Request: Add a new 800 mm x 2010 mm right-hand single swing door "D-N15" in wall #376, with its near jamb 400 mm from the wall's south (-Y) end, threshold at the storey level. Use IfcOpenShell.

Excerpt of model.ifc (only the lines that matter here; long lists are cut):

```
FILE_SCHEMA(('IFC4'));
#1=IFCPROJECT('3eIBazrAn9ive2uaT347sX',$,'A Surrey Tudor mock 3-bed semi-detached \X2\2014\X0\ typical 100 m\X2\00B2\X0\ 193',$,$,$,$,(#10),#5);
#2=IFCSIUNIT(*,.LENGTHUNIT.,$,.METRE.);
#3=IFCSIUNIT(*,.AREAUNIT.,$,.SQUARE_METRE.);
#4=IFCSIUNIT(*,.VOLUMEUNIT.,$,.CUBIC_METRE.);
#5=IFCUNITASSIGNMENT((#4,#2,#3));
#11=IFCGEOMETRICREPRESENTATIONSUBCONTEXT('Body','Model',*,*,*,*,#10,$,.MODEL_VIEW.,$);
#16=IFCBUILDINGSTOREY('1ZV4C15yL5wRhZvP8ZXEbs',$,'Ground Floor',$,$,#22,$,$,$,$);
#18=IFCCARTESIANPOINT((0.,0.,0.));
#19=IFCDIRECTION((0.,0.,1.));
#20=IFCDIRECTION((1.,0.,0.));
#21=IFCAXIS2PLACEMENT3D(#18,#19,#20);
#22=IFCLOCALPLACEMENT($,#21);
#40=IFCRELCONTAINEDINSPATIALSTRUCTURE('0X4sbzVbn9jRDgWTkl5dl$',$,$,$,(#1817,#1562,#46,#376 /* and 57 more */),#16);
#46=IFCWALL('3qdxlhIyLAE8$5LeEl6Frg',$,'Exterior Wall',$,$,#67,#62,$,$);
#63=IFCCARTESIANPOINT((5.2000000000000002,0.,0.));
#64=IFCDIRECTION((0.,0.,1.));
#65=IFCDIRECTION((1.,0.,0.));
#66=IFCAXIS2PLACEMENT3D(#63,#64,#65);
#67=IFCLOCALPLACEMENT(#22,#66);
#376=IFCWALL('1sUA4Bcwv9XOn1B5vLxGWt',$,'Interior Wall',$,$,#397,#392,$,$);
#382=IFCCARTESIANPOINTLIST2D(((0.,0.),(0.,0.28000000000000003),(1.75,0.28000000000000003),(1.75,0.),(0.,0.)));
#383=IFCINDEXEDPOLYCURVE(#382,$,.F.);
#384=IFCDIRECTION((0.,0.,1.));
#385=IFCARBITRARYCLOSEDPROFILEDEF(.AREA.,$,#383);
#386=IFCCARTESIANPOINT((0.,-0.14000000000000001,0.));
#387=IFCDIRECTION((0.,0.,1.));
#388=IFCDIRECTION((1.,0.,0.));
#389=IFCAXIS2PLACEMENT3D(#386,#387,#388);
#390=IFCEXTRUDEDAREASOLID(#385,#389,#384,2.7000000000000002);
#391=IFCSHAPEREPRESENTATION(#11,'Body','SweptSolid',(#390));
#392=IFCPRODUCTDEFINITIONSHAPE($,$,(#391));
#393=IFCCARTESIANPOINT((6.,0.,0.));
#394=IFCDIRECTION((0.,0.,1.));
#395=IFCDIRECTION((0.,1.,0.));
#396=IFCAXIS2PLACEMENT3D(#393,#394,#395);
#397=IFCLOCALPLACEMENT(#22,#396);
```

```python
import numpy as np
import ifcopenshell
import ifcopenshell.api.feature
import ifcopenshell.api.geometry
import ifcopenshell.api.root
import ifcopenshell.api.spatial
import ifcopenshell.geom
import ifcopenshell.util.element
import ifcopenshell.util.placement
import ifcopenshell.util.representation
import ifcopenshell.util.shape
import ifcopenshell.util.unit

model = ifcopenshell.open("model.ifc")
unit_scale = ifcopenshell.util.unit.calculate_unit_scale(model)
settings = ifcopenshell.geom.settings()


def volume(element):
    """Net volume in cubic metres, openings subtracted."""
    shape = ifcopenshell.geom.create_shape(settings, element)
    return ifcopenshell.util.shape.get_volume(shape.geometry)


wall = model.by_guid("1sUA4Bcwv9XOn1B5vLxGWt")
storey = ifcopenshell.util.element.get_container(wall, ifc_class="IfcBuildingStorey")
context = ifcopenshell.util.representation.get_context(model, "Model", "Body", "MODEL_VIEW")
before = volume(wall)

width, height, from_end, sill = 0.8, 2.01, 0.4, 0.0  # metres

# The wall runs along its own X axis, and the end named is its -X end.
wall_shape = ifcopenshell.geom.create_shape(settings, wall)
x, y, z = ifcopenshell.util.shape.get_vertices(wall_shape.geometry).T
start = x.min() + from_end
face, thickness = float(y.min()), float(y.max() - y.min())
wall_matrix = ifcopenshell.util.placement.get_local_placement(wall.ObjectPlacement)
level = ifcopenshell.util.placement.get_local_placement(storey.ObjectPlacement)[2, 3]


def in_wall(x, y):
    """Placement at x, y metres in the wall's axes, at sill height."""
    matrix = wall_matrix.copy()
    matrix[:, 3] = wall_matrix @ np.array([x / unit_scale, y / unit_scale, 0.0, 1.0])
    matrix[2, 3] = level + sill / unit_scale
    return matrix


# Opening: a box that overshoots both wall faces by 50 mm.
opening = ifcopenshell.api.root.create_entity(model, ifc_class="IfcOpeningElement", predefined_type="OPENING")
box = ifcopenshell.api.geometry.add_wall_representation(
    model, context=context, length=width, height=height, thickness=thickness + 0.1
)
ifcopenshell.api.geometry.assign_representation(model, product=opening, representation=box)
ifcopenshell.api.geometry.edit_object_placement(model, product=opening, matrix=in_wall(start, face - 0.05), is_si=False)
ifcopenshell.api.feature.add_feature(model, feature=opening, element=wall)

door = ifcopenshell.api.root.create_entity(model, ifc_class="IfcDoor", name="D-N15", predefined_type="DOOR")
door.OverallWidth, door.OverallHeight = width / unit_scale, height / unit_scale
door.OperationType = "SINGLE_SWING_RIGHT"
body = ifcopenshell.api.geometry.add_door_representation(
    model,
    context=context,
    overall_width=door.OverallWidth,
    overall_height=door.OverallHeight,
    operation_type="SINGLE_SWING_RIGHT",
    lining_properties={"LiningDepth": thickness / unit_scale, "ThresholdDepth": thickness / unit_scale},
)
ifcopenshell.api.geometry.assign_representation(model, product=door, representation=body)
ifcopenshell.api.spatial.assign_container(model, products=[door], relating_structure=storey)
ifcopenshell.api.feature.add_filling(model, opening=opening, element=door)

# The lining spans the wall, so the door starts at the wall face.
ifcopenshell.api.geometry.edit_object_placement(model, product=door, matrix=in_wall(start, face), is_si=False)

after = volume(wall)

print(f"wall volume {before:.3f} -> {after:.3f} m3")

model.write("model_v2.ifc")
```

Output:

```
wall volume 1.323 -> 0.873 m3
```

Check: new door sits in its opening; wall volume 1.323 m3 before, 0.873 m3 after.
